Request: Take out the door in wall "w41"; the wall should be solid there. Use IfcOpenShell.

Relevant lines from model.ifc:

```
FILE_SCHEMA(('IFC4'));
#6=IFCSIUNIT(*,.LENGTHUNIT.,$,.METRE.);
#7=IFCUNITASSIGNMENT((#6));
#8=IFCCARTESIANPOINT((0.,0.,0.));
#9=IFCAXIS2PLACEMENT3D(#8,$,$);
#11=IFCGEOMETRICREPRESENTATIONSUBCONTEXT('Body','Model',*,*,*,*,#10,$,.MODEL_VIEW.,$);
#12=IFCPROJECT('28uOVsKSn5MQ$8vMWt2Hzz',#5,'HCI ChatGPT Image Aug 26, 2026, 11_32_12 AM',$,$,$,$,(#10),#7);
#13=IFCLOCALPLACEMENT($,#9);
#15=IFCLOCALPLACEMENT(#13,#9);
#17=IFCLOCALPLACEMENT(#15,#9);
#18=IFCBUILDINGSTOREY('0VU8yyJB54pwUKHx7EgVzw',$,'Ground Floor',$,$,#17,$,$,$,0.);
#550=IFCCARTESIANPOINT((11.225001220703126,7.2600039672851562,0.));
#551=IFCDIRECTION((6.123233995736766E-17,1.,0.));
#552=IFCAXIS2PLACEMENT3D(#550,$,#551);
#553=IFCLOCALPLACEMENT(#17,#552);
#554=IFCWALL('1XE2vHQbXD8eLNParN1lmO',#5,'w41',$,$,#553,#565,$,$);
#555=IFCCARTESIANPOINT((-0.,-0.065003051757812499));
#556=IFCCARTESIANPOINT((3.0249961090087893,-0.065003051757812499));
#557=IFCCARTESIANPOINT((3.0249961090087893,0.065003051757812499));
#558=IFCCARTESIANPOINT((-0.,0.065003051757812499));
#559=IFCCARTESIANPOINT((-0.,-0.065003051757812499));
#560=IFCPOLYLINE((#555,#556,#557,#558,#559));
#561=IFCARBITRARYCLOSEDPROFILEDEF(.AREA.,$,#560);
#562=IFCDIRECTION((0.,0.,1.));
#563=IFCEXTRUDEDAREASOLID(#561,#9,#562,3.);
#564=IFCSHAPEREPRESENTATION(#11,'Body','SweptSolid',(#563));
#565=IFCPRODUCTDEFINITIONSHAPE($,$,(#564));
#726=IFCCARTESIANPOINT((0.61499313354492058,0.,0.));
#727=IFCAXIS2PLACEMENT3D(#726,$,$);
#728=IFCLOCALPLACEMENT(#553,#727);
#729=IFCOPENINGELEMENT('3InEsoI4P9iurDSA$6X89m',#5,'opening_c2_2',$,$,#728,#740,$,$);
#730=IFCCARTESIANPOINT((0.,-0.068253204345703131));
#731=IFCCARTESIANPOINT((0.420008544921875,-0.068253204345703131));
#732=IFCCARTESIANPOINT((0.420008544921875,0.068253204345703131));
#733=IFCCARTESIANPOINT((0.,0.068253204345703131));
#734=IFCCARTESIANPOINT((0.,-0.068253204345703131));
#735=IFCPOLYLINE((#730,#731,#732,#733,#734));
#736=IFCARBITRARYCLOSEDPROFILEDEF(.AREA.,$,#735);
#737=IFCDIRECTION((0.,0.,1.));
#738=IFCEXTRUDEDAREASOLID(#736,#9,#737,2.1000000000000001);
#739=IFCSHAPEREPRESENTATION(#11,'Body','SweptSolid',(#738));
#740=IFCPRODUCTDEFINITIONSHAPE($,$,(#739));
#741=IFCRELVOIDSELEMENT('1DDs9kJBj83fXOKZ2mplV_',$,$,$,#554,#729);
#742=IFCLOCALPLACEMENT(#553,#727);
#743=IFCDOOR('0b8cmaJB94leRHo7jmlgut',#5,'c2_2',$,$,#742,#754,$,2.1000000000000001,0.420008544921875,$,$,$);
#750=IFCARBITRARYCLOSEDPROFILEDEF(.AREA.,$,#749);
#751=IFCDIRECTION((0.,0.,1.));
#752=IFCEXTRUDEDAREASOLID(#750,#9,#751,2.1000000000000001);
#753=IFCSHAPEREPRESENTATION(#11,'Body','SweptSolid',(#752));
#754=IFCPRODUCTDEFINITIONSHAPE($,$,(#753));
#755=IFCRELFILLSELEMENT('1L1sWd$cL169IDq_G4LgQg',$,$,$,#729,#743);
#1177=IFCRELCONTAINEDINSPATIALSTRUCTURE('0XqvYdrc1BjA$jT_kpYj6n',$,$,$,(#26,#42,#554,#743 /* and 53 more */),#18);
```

```python
import ifcopenshell
import ifcopenshell.api.feature
import ifcopenshell.api.root
import ifcopenshell.geom
import ifcopenshell.util.shape

model = ifcopenshell.open("model.ifc")
settings = ifcopenshell.geom.settings()


def volume(element):
    """Net volume in cubic metres, openings subtracted."""
    shape = ifcopenshell.geom.create_shape(settings, element)
    return ifcopenshell.util.shape.get_volume(shape.geometry)


door = model.by_id(743)
opening = door.FillsVoids[0].RelatingOpeningElement
wall = opening.VoidsElements[0].RelatingBuildingElement
before = volume(wall)

ifcopenshell.api.root.remove_product(model, product=door)
ifcopenshell.api.feature.remove_feature(model, feature=opening)

after = volume(wall)

print(f"wall volume {before:.3f} -> {after:.3f} m3")

model.write("model_edited.ifc")
```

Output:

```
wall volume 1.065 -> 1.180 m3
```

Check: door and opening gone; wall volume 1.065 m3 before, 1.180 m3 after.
